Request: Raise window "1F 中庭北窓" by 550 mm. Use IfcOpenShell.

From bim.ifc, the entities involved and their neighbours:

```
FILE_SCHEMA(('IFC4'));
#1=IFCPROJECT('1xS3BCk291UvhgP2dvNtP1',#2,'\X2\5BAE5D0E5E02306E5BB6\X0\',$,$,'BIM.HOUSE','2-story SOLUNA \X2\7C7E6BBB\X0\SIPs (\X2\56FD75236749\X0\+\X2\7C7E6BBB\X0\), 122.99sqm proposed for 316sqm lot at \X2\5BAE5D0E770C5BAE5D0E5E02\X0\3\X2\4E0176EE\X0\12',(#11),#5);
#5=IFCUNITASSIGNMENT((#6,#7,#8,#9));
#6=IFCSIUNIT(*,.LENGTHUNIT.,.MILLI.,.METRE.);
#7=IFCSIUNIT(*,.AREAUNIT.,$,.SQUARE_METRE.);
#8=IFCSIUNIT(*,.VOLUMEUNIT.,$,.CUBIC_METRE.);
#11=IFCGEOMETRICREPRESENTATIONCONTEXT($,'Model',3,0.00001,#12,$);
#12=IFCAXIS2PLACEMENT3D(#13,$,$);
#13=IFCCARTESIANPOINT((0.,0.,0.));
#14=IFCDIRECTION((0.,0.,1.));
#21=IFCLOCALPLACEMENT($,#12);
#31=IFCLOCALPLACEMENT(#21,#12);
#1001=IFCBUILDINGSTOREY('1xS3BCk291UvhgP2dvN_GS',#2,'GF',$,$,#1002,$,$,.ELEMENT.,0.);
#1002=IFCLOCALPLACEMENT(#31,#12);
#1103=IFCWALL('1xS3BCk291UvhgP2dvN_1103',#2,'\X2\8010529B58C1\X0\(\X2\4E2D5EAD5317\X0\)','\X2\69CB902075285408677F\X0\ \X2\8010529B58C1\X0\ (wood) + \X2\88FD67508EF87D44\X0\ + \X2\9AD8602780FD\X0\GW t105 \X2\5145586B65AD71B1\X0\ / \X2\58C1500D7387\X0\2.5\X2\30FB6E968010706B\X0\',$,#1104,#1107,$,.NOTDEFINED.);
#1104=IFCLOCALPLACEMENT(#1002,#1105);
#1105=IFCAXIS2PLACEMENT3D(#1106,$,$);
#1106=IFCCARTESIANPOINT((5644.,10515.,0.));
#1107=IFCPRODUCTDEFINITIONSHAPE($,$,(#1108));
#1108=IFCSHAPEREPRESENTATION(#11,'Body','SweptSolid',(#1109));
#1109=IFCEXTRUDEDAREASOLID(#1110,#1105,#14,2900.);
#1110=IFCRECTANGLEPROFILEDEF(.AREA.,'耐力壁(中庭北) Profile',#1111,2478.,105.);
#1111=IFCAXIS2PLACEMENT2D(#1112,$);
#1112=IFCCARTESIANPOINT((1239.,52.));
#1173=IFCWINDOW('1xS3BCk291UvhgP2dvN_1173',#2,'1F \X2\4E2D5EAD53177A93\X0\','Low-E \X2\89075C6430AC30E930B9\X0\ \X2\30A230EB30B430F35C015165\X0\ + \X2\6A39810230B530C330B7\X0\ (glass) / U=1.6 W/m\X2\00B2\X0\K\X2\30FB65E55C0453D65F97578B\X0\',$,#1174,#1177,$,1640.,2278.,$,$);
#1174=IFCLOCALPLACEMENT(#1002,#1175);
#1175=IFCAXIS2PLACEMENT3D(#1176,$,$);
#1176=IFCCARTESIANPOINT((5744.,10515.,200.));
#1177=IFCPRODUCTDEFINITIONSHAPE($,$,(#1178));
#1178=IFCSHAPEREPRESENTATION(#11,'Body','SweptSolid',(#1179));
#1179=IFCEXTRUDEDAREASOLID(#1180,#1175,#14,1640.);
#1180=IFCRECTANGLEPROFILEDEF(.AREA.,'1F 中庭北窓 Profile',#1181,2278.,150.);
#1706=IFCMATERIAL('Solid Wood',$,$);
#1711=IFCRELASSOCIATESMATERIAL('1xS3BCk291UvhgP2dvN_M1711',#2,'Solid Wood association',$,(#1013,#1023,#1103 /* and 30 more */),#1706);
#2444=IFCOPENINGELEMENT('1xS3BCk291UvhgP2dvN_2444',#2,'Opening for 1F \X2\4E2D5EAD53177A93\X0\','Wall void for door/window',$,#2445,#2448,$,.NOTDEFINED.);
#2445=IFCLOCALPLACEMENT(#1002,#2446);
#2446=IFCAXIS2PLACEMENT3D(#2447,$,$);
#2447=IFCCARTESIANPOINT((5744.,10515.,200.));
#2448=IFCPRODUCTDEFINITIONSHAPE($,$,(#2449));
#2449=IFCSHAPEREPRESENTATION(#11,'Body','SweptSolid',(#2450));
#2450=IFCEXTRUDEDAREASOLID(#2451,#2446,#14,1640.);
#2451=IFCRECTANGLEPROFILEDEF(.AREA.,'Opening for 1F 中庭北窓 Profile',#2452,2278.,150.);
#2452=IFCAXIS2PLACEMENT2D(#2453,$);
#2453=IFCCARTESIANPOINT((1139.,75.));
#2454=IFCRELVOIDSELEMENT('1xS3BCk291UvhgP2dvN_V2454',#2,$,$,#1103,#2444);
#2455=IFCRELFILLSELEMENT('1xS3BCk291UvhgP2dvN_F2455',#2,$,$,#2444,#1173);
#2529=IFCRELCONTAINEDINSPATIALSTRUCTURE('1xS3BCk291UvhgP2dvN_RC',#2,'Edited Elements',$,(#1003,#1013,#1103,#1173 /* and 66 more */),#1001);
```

```python
import numpy as np
import ifcopenshell
import ifcopenshell.api.geometry
import ifcopenshell.util.placement
import ifcopenshell.util.unit

model = ifcopenshell.open("bim.ifc")
unit_scale = ifcopenshell.util.unit.calculate_unit_scale(model)

window = model.by_guid("1xS3BCk291UvhgP2dvN_1173")
opening = window.FillsVoids[0].RelatingOpeningElement
dz = 550.0

shift = np.array([0.0, 0.0, dz])
# The window is not placed relative to its opening, so move both.
for product in (opening, window):
    matrix = ifcopenshell.util.placement.get_local_placement(product.ObjectPlacement)
    matrix[:3, 3] += shift
    ifcopenshell.api.geometry.edit_object_placement(model, product=product, matrix=matrix, is_si=False)

print(f"moved by {dz * unit_scale:+.3f} m")

model.write("bim-out.ifc")
```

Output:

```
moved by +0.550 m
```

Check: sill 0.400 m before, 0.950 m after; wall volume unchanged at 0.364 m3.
